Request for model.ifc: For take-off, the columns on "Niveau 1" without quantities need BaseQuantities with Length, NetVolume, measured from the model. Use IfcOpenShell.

First a look at what the model holds.

```python
import ifcopenshell
import ifcopenshell.util.element
import ifcopenshell.util.unit

model = ifcopenshell.open("model.ifc")
print(model.schema)
for unit_type in ("LENGTHUNIT", "AREAUNIT", "VOLUMEUNIT"):
    print(unit_type, ifcopenshell.util.unit.calculate_unit_scale(model, unit_type))
storey = next(s for s in model.by_type("IfcBuildingStorey") if s.Name == "Niveau 1")
columns = [e for e in ifcopenshell.util.element.get_decomposition(storey) if e.is_a("IfcColumn")]
for e in sorted(columns, key=lambda e: e.id()):
    print(e.id(), e.is_a(), e.Name, list(ifcopenshell.util.element.get_psets(e, qtos_only=True)), sep=" | ")
```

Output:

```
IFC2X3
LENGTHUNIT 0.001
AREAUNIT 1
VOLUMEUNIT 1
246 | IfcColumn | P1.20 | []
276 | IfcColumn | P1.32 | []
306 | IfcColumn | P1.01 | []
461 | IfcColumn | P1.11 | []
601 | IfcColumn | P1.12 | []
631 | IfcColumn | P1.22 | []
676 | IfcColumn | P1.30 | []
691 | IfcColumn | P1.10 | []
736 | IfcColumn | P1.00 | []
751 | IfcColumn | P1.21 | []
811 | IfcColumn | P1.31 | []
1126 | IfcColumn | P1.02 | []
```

```python
import ifcopenshell
import ifcopenshell.api.pset
import ifcopenshell.geom
import ifcopenshell.util.element
import ifcopenshell.util.shape
import ifcopenshell.util.unit

model = ifcopenshell.open("model.ifc")
unit_scale = ifcopenshell.util.unit.calculate_unit_scale(model)
volume_scale = ifcopenshell.util.unit.calculate_unit_scale(model, "VOLUMEUNIT")
settings = ifcopenshell.geom.settings()

storey = next(s for s in model.by_type("IfcBuildingStorey") if s.Name == "Niveau 1")
columns = [e for e in ifcopenshell.util.element.get_decomposition(storey) if e.is_a("IfcColumn")]

for e in sorted(columns, key=lambda e: e.id()):
    if ifcopenshell.util.element.get_psets(e, qtos_only=True, should_inherit=False):
        continue
    # Geometry comes back in metres, in the element's own axes.
    shape = ifcopenshell.geom.create_shape(settings, e)
    values = {
        "Length": ifcopenshell.util.shape.get_z(shape.geometry) / unit_scale,
        "NetVolume": ifcopenshell.util.shape.get_volume(shape.geometry) / volume_scale,
    }
    qto = ifcopenshell.api.pset.add_qto(model, product=e, name="BaseQuantities")
    ifcopenshell.api.pset.edit_qto(model, qto=qto, properties=values)
    print(e.id(), {k: round(v, 3) for k, v in values.items()})

model.write("model_v2.ifc")
```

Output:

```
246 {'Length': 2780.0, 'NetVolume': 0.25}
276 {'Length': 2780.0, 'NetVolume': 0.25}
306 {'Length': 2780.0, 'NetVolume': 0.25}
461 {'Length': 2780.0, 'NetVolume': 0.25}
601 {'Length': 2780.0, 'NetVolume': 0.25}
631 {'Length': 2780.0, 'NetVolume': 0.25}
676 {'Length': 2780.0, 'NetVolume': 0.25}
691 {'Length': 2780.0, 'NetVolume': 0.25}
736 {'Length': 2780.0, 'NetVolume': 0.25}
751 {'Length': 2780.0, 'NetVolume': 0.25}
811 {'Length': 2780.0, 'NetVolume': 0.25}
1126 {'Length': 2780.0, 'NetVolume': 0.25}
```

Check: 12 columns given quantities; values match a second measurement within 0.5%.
